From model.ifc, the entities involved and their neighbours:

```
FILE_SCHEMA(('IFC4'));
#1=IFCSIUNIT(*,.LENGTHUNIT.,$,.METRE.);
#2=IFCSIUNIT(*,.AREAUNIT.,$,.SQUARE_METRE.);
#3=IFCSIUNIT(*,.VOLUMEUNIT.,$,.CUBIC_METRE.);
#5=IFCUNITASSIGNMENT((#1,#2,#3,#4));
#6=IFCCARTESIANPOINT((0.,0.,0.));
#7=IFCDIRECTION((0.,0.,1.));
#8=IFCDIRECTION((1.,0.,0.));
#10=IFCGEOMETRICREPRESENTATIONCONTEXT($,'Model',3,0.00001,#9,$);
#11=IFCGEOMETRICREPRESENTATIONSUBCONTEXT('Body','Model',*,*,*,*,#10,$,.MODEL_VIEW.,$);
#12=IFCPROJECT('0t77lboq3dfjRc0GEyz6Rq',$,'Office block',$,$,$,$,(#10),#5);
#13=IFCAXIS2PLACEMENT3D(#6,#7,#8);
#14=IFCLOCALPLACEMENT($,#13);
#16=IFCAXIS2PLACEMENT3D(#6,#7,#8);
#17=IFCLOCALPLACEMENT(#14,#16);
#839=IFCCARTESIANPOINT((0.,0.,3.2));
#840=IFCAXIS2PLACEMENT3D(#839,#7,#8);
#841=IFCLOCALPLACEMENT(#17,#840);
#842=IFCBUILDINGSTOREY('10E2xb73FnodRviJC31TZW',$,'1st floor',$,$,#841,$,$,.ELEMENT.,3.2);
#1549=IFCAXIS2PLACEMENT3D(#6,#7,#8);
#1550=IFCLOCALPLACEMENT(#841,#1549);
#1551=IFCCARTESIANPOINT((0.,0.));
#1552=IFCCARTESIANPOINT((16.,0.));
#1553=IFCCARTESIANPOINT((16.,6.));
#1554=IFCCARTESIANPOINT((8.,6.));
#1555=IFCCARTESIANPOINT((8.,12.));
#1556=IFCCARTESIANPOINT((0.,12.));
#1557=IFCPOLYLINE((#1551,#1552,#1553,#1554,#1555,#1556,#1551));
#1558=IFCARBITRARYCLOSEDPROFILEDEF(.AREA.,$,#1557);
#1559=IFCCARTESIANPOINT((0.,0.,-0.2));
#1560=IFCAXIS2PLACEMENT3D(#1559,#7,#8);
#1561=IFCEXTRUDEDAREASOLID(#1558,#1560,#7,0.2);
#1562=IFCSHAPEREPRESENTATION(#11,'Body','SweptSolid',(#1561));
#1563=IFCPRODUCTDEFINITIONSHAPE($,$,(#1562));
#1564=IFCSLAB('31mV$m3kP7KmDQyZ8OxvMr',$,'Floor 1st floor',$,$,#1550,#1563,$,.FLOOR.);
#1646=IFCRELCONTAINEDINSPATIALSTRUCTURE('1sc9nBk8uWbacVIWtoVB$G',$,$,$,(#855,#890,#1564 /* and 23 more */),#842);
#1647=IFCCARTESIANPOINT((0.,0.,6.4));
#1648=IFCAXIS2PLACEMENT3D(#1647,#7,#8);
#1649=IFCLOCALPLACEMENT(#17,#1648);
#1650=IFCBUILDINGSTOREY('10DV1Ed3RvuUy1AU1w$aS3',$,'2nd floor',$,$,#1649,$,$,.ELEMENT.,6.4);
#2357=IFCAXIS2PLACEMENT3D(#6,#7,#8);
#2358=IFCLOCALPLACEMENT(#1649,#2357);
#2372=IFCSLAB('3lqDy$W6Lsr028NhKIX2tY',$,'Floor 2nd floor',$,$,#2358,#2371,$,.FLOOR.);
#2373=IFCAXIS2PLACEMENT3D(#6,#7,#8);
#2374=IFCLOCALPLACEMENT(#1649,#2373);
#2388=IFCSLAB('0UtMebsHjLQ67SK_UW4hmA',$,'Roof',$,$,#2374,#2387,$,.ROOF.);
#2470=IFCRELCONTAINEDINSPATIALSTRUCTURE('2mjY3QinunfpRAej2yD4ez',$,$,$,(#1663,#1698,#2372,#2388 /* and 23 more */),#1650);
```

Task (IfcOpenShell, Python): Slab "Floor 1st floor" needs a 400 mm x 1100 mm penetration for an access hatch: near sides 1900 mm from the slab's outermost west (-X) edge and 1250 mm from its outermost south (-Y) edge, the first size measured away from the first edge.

```python
import numpy as np
import ifcopenshell
import ifcopenshell.api.feature
import ifcopenshell.api.geometry
import ifcopenshell.api.root
import ifcopenshell.geom
import ifcopenshell.util.placement
import ifcopenshell.util.representation
import ifcopenshell.util.shape
import ifcopenshell.util.unit

model = ifcopenshell.open("model.ifc")
unit_scale = ifcopenshell.util.unit.calculate_unit_scale(model)
settings = ifcopenshell.geom.settings()


def volume(element):
    """Net volume in cubic metres, openings subtracted."""
    shape = ifcopenshell.geom.create_shape(settings, element)
    return ifcopenshell.util.shape.get_volume(shape.geometry)


slab = model.by_guid("31mV$m3kP7KmDQyZ8OxvMr")
before = volume(slab)

# Extent in the slab's own axes, in metres. The edges named are its -X and -Y sides.
slab_shape = ifcopenshell.geom.create_shape(settings, slab)
vertices = ifcopenshell.util.shape.get_vertices(slab_shape.geometry)
x_min, y_min, bottom = vertices.min(axis=0)
top = vertices[:, 2].max()

opening = ifcopenshell.api.root.create_entity(model, ifc_class="IfcOpeningElement", name="Access hatch opening", predefined_type="OPENING")
context = ifcopenshell.util.representation.get_context(model, "Model", "Body", "MODEL_VIEW")
width, depth = 0.4, 1.1
outline = [(0.0, 0.0), (width, 0.0), (width, depth), (0.0, depth), (0.0, 0.0)]
# Overshoot both faces by 50 mm so the cut is clean.
shape = ifcopenshell.api.geometry.add_slab_representation(
    model, context=context, depth=top - bottom + 0.1, polyline=outline
)
ifcopenshell.api.geometry.assign_representation(model, product=opening, representation=shape)

matrix = ifcopenshell.util.placement.get_local_placement(slab.ObjectPlacement)
matrix[:, 3] = matrix @ np.append(np.array([x_min + 1.9, y_min + 1.25, bottom - 0.05]) / unit_scale, 1.0)
ifcopenshell.api.geometry.edit_object_placement(model, product=opening, matrix=matrix, is_si=False)
ifcopenshell.api.feature.add_feature(model, feature=opening, element=slab)

after = volume(slab)

print(f"slab volume {before:.3f} -> {after:.3f} m3")

model.write("model_v2.ifc")
```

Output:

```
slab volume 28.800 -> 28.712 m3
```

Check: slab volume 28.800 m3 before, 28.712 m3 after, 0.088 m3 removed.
